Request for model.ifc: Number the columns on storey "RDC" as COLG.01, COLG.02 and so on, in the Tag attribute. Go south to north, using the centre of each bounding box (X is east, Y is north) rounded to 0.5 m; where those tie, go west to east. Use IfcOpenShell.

First a look at what the model holds.

```python
import ifcopenshell
import ifcopenshell.util.element
import ifcopenshell.util.placement

model = ifcopenshell.open("model.ifc")
print(model.schema)
storey = next(s for s in model.by_type("IfcBuildingStorey") if s.Name == "RDC")
columns = [e for e in ifcopenshell.util.element.get_decomposition(storey) if e.is_a("IfcColumn")]
for e in sorted(columns, key=lambda e: e.id()):
    origin = ifcopenshell.util.placement.get_local_placement(e.ObjectPlacement)[:3, 3]
    print(e.id(), e.Tag, e.Name, origin.round(2) + 0.0, sep=" | ")
```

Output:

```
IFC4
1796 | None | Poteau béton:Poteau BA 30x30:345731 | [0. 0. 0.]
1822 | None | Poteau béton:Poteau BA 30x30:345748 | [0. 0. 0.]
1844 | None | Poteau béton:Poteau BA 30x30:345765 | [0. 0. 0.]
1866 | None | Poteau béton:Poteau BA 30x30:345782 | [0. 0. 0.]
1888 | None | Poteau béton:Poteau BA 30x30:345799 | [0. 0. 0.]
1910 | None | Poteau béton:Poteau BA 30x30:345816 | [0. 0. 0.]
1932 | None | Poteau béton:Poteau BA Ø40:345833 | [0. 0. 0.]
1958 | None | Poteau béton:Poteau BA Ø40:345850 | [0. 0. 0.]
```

```python
import ifcopenshell
import ifcopenshell.geom
import ifcopenshell.util.element
import ifcopenshell.util.shape

model = ifcopenshell.open("model.ifc")
settings = ifcopenshell.geom.settings()
settings.set("use-world-coords", True)


def centre(element):
    shape = ifcopenshell.geom.create_shape(settings, element)
    return ifcopenshell.util.shape.get_bbox_centroid(shape.geometry)


storey = next(s for s in model.by_type("IfcBuildingStorey") if s.Name == "RDC")
columns = [e for e in ifcopenshell.util.element.get_decomposition(storey) if e.is_a("IfcColumn")]

# Insertion points can sit at a corner or the storey origin, so sort by the geometry (in metres).
centres = {e: centre(e) for e in columns}
columns.sort(key=lambda e: (round(centres[e][1] / 0.5), centres[e][0]))

for i, e in enumerate(columns, start=1):
    number = f"COLG.{i:02d}"
    e.Tag = number
    print(e.id(), number)

model.write("model_edited.ifc")
```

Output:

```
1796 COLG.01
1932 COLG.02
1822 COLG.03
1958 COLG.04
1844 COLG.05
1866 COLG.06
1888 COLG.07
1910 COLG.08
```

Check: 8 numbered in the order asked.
